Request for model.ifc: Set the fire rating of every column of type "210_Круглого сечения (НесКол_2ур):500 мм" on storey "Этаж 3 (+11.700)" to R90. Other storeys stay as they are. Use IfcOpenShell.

First a look at what the model holds.

```python
import ifcopenshell
import ifcopenshell.util.element

model = ifcopenshell.open("model.ifc")
print(model.schema)
storey = next(s for s in model.by_type("IfcBuildingStorey") if s.Name == "Этаж 3 (+11.700)")
columns = [e for e in ifcopenshell.util.element.get_decomposition(storey) if e.is_a("IfcColumn")]
seen = {}
for e in columns:
    element_type = ifcopenshell.util.element.get_type(e)
    key = (element_type.Name if element_type != e and element_type else None, ifcopenshell.util.element.get_pset(e, "Pset_ColumnCommon", "FireRating"))
    seen[key] = seen.get(key, 0) + 1
for (name, value), count in sorted(seen.items(), key=str):
    print(count, "x", name, "|", value)
```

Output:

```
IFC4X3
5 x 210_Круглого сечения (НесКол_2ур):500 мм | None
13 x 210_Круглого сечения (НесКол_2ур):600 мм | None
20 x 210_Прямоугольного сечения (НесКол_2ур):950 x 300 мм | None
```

```python
import ifcopenshell
import ifcopenshell.api.pset
import ifcopenshell.util.element

model = ifcopenshell.open("model.ifc")

storey = next(s for s in model.by_type("IfcBuildingStorey") if s.Name == "Этаж 3 (+11.700)")
columns = [e for e in ifcopenshell.util.element.get_decomposition(storey) if e.is_a("IfcColumn")]

count = 0
for e in columns:
    element_type = ifcopenshell.util.element.get_type(e)
    if element_type in (None, e) or element_type.Name != "210_Круглого сечения (НесКол_2ур):500 мм":
        continue
    # add_pset returns the element's existing set when there is one.
    pset = ifcopenshell.api.pset.add_pset(model, product=e, name="Pset_ColumnCommon")
    ifcopenshell.api.pset.edit_pset(model, pset=pset, properties={"FireRating": "R90"})
    count += 1

print(count, "columns updated")

model.write("model_updated.ifc")
```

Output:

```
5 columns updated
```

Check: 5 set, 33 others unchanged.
